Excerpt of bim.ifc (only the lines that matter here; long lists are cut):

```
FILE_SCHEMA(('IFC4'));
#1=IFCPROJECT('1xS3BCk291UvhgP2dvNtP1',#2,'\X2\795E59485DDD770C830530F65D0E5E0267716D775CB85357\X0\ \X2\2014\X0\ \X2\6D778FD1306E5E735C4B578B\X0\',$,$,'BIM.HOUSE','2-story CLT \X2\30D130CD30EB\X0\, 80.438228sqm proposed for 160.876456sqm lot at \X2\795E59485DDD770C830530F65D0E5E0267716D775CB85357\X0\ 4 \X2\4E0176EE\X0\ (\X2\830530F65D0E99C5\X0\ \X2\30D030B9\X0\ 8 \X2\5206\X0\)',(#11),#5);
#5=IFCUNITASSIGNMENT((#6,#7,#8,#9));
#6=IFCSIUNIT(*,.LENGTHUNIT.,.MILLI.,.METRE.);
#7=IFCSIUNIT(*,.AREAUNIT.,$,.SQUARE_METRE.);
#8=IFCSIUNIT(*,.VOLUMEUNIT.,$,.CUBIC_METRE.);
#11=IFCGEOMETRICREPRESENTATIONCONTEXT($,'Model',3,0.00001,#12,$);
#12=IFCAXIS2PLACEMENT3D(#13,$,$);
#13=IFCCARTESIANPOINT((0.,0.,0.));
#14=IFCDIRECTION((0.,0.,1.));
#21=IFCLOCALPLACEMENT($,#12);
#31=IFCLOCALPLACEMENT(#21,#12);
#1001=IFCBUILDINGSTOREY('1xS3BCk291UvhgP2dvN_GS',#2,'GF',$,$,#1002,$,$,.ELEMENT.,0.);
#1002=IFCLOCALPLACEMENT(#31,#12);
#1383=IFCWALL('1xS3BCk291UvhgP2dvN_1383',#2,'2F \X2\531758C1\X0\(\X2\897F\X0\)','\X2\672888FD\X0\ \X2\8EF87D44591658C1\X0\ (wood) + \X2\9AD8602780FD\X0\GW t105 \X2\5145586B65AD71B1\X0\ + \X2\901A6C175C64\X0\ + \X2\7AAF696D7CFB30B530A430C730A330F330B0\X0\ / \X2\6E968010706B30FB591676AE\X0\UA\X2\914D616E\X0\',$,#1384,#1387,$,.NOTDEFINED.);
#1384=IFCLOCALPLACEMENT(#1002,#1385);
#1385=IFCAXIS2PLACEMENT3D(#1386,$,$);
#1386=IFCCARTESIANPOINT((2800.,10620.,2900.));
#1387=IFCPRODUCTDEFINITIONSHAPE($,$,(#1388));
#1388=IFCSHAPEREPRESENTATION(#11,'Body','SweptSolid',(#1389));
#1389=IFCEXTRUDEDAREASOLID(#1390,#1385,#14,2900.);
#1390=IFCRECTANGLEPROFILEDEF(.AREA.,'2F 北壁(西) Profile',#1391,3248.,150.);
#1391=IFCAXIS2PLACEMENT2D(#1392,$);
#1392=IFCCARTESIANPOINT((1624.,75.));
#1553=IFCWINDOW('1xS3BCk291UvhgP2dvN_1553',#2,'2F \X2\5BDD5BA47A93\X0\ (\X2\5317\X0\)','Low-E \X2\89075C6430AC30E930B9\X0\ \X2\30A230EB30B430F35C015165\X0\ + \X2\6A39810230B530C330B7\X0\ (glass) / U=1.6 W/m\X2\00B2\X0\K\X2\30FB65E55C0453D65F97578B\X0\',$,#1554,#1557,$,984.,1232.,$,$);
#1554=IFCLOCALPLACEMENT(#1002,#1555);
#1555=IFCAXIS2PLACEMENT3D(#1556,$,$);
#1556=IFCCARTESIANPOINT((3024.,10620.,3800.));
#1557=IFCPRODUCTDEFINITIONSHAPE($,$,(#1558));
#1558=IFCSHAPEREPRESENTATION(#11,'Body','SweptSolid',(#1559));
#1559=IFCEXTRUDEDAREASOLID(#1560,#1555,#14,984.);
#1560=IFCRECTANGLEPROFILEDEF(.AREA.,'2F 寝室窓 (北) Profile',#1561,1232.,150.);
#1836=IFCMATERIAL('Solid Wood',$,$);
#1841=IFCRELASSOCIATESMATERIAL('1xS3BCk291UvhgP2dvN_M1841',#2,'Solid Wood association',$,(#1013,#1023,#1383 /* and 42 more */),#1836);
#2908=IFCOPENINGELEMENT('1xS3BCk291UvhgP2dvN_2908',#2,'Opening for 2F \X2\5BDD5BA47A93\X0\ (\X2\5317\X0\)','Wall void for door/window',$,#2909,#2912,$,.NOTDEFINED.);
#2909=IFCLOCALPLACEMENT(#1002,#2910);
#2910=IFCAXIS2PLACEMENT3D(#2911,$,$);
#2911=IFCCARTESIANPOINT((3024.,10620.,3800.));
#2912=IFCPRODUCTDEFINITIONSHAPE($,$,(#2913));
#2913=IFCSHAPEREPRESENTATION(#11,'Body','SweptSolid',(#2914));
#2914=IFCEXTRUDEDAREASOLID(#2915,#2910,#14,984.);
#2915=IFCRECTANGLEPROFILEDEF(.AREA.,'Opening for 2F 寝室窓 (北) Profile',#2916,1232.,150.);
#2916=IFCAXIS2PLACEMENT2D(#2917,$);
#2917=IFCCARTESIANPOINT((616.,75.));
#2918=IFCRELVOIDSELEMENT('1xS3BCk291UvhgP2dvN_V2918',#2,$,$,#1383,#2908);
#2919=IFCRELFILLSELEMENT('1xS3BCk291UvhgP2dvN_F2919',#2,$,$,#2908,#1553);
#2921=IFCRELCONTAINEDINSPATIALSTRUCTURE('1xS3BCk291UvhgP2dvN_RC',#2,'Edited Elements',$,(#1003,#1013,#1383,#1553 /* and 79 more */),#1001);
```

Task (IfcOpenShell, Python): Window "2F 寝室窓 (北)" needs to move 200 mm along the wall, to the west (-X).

```python
import ifcopenshell
import ifcopenshell.api.geometry
import ifcopenshell.util.placement

model = ifcopenshell.open("bim.ifc")

window = model.by_id(1553)
opening = window.FillsVoids[0].RelatingOpeningElement
wall = opening.VoidsElements[0].RelatingBuildingElement

wall_matrix = ifcopenshell.util.placement.get_local_placement(wall.ObjectPlacement)
shift = wall_matrix[:3, 0] * -200.0
before = ifcopenshell.util.placement.get_local_placement(window.ObjectPlacement)[:3, 3].copy()

# The window is not placed relative to its opening, so move both.
for product in (opening, window):
    matrix = ifcopenshell.util.placement.get_local_placement(product.ObjectPlacement)
    matrix[:3, 3] += shift
    ifcopenshell.api.geometry.edit_object_placement(model, product=product, matrix=matrix, is_si=False)

after = ifcopenshell.util.placement.get_local_placement(window.ObjectPlacement)[:3, 3]
print("window moved by", (after - before).round(3) + 0.0)

model.write("bim-out.ifc")
```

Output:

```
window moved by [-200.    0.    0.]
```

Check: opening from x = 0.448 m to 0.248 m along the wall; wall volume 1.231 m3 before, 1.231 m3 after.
